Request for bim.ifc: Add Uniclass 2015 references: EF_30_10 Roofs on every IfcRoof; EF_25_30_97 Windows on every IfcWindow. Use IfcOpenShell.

First a look at what the model holds.

```python
import ifcopenshell

model = ifcopenshell.open("bim.ifc")
print(model.schema)
print("classifications:", [c.Name for c in model.by_type("IfcClassification")])
for ifc_class in ("IfcDoor", "IfcRoof", "IfcStair", "IfcWall", "IfcWindow"):
    print(ifc_class, len(model.by_type(ifc_class)))
```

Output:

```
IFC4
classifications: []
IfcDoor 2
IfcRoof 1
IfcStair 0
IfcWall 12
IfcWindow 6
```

```python
import ifcopenshell
import ifcopenshell.api.classification

model = ifcopenshell.open("bim.ifc")

system = ifcopenshell.api.classification.add_classification(model, classification="Uniclass 2015")

codes = {
    "IfcRoof": ("EF_30_10", "Roofs"),
    "IfcWindow": ("EF_25_30_97", "Windows"),
}
for ifc_class, (code, name) in codes.items():
    products = model.by_type(ifc_class)
    ifcopenshell.api.classification.add_reference(
        model, products=products, classification=system, identification=code, name=name
    )
    print(code, len(products))

model.write("bim_updated.ifc")
```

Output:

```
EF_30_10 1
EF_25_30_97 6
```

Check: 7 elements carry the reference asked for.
